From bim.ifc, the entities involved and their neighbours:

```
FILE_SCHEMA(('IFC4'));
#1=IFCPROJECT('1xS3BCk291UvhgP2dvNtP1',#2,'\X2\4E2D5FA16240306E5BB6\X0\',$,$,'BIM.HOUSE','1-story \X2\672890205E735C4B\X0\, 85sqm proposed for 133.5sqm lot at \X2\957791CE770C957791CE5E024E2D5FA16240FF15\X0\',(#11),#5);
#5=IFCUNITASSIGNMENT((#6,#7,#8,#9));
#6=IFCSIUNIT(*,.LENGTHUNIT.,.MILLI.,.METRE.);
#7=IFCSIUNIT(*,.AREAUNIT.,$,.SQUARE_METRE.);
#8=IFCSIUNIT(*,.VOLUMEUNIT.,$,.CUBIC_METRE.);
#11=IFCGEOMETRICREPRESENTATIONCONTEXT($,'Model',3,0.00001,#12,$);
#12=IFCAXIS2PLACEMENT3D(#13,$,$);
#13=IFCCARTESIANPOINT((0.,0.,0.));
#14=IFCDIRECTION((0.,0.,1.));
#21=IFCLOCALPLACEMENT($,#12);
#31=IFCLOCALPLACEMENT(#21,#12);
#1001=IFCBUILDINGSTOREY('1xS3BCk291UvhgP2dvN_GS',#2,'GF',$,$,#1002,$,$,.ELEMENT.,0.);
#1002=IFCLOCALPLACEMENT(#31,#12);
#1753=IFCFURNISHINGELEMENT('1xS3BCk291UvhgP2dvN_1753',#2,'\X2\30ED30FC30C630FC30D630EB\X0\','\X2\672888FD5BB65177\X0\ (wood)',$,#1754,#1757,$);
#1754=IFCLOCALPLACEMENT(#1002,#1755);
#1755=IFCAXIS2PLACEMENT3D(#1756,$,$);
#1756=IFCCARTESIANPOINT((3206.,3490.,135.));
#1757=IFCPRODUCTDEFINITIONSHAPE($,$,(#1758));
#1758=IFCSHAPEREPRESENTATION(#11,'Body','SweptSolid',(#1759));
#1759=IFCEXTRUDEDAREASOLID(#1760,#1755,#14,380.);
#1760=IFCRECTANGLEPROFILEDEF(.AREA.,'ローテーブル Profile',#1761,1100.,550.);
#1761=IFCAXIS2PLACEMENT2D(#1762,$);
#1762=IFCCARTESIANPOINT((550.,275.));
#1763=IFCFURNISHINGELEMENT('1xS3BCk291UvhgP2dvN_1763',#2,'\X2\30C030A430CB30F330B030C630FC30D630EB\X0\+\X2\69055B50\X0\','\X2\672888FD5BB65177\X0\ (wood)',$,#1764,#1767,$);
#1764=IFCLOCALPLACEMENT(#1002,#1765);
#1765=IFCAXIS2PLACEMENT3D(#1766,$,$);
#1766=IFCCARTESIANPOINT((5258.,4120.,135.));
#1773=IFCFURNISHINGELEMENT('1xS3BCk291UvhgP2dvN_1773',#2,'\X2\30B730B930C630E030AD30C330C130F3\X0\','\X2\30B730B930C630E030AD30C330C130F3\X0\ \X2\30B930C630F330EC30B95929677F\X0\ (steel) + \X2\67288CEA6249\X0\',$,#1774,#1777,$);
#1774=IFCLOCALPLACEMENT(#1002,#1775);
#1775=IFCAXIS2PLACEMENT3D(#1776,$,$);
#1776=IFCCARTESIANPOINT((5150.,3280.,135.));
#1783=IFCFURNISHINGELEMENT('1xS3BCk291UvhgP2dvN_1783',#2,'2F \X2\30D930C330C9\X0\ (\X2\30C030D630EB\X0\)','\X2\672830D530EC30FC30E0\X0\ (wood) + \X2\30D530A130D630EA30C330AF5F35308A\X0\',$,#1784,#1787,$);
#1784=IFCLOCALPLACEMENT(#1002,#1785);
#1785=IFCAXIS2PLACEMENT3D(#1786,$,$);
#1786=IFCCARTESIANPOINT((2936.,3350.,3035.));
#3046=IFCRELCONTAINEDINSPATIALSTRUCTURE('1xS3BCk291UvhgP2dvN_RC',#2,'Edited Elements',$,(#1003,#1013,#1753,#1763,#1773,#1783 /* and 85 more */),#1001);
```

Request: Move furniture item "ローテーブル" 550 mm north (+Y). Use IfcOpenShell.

```python
import ifcopenshell
import ifcopenshell.api.geometry
import ifcopenshell.util.placement
import ifcopenshell.util.unit

model = ifcopenshell.open("bim.ifc")
unit_scale = ifcopenshell.util.unit.calculate_unit_scale(model)

item = model.by_guid("1xS3BCk291UvhgP2dvN_1753")
matrix = ifcopenshell.util.placement.get_local_placement(item.ObjectPlacement)
matrix[1, 3] += 0.55 / unit_scale
ifcopenshell.api.geometry.edit_object_placement(model, product=item, matrix=matrix, is_si=False)

print(ifcopenshell.util.placement.get_local_placement(item.ObjectPlacement).round(3) + 0.0)

model.write("bim_v2.ifc")
```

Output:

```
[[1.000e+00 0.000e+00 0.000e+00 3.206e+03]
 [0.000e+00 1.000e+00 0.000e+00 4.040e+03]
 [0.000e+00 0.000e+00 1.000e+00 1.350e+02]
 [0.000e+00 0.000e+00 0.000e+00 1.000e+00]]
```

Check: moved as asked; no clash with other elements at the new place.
